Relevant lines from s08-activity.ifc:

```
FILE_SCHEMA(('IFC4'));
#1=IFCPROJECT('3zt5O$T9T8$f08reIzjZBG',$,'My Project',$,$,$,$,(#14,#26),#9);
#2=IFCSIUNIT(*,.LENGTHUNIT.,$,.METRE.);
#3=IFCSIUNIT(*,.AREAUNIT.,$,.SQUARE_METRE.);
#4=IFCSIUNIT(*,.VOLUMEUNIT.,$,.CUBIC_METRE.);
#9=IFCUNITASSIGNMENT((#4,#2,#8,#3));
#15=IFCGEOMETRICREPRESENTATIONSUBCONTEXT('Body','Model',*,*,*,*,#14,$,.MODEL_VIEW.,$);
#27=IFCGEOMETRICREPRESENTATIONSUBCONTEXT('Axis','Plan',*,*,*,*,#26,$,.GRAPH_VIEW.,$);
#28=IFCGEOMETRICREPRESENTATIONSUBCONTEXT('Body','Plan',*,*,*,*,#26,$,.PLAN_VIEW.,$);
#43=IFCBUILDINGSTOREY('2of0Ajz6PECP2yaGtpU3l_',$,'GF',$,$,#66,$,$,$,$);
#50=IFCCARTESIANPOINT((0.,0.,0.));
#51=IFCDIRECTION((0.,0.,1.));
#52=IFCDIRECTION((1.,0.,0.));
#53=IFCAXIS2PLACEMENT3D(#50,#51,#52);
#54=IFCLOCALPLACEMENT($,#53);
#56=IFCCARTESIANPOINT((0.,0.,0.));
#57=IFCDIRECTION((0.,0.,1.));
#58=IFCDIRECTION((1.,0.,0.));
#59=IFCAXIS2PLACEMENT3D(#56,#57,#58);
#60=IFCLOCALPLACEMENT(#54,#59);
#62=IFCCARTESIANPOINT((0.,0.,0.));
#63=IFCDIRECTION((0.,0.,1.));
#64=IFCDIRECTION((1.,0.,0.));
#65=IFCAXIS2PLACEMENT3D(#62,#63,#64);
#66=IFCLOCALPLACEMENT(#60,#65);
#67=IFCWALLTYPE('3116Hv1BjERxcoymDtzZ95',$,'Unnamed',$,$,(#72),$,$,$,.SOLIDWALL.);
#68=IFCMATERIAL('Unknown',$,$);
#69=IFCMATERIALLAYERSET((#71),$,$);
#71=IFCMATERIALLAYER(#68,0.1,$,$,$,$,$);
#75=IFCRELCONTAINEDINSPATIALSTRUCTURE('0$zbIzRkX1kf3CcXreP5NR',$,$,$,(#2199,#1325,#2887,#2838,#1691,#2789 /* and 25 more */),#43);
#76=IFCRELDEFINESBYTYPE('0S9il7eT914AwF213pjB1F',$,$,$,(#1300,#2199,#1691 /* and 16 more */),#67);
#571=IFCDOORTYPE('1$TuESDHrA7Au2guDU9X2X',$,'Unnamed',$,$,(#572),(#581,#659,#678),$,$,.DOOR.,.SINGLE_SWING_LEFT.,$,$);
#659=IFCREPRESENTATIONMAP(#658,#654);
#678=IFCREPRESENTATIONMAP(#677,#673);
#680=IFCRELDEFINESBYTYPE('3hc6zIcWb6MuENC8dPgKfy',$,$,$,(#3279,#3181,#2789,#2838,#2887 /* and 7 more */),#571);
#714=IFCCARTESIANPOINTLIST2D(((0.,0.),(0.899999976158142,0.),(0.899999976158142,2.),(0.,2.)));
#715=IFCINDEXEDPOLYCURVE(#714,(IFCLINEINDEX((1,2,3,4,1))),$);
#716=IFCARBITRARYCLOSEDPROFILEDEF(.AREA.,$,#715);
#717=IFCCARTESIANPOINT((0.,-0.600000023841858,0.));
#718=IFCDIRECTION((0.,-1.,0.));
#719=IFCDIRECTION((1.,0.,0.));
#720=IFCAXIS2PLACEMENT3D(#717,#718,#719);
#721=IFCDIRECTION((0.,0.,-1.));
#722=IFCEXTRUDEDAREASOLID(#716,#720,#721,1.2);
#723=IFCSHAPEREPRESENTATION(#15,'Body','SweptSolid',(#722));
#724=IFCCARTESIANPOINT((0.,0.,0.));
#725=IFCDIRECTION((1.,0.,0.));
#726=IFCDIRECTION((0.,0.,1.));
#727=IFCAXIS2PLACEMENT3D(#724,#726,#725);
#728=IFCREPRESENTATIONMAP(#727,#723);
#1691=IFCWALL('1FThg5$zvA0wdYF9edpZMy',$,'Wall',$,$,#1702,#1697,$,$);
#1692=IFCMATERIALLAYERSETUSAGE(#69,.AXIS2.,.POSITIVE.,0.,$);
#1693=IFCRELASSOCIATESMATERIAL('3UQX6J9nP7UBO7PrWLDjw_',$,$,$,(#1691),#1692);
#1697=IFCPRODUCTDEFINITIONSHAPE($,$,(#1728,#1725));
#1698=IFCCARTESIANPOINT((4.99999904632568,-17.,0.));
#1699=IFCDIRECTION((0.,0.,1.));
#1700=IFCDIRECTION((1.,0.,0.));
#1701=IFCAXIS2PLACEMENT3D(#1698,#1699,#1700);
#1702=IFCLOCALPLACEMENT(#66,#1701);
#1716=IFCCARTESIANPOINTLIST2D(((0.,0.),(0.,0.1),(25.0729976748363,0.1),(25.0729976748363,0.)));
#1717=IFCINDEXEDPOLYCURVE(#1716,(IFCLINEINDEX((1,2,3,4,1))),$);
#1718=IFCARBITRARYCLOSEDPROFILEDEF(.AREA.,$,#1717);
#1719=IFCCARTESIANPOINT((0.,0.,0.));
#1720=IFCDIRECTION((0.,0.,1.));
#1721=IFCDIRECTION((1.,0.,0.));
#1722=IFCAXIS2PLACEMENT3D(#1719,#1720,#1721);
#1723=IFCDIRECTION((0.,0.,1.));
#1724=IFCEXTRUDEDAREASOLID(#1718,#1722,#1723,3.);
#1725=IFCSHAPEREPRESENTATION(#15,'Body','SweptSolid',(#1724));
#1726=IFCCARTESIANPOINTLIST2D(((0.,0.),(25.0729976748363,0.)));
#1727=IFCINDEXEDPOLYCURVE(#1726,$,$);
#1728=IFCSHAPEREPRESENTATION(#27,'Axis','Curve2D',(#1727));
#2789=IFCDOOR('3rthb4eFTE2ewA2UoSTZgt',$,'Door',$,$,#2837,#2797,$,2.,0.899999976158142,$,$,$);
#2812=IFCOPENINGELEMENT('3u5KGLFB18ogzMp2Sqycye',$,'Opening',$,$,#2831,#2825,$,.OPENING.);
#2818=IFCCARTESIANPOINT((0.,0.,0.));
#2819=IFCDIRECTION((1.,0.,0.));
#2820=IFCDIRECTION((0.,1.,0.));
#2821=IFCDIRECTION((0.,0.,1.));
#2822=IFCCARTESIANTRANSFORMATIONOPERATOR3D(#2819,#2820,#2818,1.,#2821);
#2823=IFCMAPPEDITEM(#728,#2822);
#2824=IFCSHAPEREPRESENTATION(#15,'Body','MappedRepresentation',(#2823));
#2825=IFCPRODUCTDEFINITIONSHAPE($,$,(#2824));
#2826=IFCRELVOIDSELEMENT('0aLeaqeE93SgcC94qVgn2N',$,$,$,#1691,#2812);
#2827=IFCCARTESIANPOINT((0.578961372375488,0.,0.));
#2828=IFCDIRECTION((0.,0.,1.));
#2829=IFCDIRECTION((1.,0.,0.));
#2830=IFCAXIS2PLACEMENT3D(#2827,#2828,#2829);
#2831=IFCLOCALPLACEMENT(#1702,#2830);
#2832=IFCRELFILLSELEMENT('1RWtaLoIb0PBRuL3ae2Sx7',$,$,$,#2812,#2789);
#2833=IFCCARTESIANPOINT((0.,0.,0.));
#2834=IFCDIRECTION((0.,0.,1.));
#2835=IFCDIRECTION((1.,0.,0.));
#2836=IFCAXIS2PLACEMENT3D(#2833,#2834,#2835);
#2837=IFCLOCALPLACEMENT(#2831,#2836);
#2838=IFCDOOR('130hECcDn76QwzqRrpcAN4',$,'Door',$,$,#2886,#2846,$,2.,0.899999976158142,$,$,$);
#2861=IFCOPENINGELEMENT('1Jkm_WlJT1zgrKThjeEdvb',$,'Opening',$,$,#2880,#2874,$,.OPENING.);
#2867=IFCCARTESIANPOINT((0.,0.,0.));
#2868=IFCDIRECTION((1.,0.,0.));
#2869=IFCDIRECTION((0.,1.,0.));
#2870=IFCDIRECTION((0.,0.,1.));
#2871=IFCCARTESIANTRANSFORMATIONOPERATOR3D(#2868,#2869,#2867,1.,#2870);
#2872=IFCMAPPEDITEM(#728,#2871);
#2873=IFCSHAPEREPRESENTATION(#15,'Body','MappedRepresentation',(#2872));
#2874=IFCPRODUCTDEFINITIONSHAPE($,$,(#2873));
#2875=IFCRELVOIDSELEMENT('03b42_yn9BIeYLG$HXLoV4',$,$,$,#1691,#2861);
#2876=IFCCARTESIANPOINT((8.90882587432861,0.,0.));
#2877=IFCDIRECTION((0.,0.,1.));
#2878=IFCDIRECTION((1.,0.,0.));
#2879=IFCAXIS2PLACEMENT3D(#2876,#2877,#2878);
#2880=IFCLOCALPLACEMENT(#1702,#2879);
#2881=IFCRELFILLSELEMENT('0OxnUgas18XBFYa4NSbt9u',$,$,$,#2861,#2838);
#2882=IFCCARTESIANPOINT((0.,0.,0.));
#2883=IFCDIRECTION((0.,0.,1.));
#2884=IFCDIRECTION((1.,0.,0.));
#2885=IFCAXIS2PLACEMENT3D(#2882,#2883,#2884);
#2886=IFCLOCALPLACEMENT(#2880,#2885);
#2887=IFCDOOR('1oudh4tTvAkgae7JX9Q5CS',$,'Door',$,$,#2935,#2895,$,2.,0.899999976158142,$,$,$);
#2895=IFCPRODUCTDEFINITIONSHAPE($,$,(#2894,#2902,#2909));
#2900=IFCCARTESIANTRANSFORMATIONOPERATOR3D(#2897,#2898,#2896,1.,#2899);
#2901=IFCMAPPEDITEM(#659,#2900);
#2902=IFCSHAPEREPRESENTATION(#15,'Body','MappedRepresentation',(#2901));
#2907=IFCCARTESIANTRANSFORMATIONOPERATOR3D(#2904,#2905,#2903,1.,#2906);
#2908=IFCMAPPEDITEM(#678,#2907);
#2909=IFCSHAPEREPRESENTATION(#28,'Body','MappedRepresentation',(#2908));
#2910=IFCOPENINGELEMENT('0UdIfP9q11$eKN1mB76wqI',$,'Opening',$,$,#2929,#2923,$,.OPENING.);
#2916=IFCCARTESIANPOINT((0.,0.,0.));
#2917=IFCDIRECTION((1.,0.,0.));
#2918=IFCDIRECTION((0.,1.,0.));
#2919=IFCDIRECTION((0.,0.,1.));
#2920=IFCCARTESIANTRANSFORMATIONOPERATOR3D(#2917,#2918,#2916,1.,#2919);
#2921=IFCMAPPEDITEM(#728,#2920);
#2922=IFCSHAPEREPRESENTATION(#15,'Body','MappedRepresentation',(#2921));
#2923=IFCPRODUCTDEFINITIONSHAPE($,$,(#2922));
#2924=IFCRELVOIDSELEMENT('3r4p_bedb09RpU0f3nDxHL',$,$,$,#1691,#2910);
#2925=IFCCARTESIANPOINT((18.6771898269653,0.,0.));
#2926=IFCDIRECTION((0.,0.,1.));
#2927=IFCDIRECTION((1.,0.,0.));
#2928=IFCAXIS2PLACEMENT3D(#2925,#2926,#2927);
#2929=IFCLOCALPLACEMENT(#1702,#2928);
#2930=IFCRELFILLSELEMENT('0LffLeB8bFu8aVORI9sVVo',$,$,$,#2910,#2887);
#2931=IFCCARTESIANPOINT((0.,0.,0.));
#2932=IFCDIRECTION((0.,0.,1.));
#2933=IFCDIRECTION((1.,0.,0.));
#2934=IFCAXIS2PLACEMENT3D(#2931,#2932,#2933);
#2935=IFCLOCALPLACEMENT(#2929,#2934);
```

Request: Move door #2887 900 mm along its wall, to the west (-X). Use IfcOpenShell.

```python
import ifcopenshell
import ifcopenshell.api.geometry
import ifcopenshell.util.placement
import ifcopenshell.util.unit

model = ifcopenshell.open("s08-activity.ifc")
unit_scale = ifcopenshell.util.unit.calculate_unit_scale(model)

door = model.by_guid("1oudh4tTvAkgae7JX9Q5CS")
opening = door.FillsVoids[0].RelatingOpeningElement
wall = opening.VoidsElements[0].RelatingBuildingElement

wall_matrix = ifcopenshell.util.placement.get_local_placement(wall.ObjectPlacement)
shift = wall_matrix[:3, 0] * -0.9 / unit_scale
before = ifcopenshell.util.placement.get_local_placement(door.ObjectPlacement)[:3, 3].copy()

# The door is placed relative to its opening, so it follows when the opening moves.
matrix = ifcopenshell.util.placement.get_local_placement(opening.ObjectPlacement)
matrix[:3, 3] += shift
ifcopenshell.api.geometry.edit_object_placement(
    model, product=opening, matrix=matrix, is_si=False, should_transform_children=True
)

after = ifcopenshell.util.placement.get_local_placement(door.ObjectPlacement)[:3, 3]
print("door moved by", (after - before).round(3) + 0.0)

model.write("s08-activity_rev.ifc")
```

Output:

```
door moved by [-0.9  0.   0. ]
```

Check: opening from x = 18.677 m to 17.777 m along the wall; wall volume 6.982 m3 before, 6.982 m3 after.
